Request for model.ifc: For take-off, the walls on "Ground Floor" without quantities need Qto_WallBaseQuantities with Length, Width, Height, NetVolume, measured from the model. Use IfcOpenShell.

First a look at what the model holds.

```python
import ifcopenshell
import ifcopenshell.util.element
import ifcopenshell.util.unit

model = ifcopenshell.open("model.ifc")
print(model.schema)
for unit_type in ("LENGTHUNIT", "AREAUNIT", "VOLUMEUNIT"):
    print(unit_type, ifcopenshell.util.unit.calculate_unit_scale(model, unit_type))
storey = next(s for s in model.by_type("IfcBuildingStorey") if s.Name == "Ground Floor")
walls = [e for e in ifcopenshell.util.element.get_decomposition(storey) if e.is_a("IfcWall")]
for e in sorted(walls, key=lambda e: e.id()):
    print(e.id(), e.is_a(), e.Name, list(ifcopenshell.util.element.get_psets(e, qtos_only=True)), sep=" | ")
```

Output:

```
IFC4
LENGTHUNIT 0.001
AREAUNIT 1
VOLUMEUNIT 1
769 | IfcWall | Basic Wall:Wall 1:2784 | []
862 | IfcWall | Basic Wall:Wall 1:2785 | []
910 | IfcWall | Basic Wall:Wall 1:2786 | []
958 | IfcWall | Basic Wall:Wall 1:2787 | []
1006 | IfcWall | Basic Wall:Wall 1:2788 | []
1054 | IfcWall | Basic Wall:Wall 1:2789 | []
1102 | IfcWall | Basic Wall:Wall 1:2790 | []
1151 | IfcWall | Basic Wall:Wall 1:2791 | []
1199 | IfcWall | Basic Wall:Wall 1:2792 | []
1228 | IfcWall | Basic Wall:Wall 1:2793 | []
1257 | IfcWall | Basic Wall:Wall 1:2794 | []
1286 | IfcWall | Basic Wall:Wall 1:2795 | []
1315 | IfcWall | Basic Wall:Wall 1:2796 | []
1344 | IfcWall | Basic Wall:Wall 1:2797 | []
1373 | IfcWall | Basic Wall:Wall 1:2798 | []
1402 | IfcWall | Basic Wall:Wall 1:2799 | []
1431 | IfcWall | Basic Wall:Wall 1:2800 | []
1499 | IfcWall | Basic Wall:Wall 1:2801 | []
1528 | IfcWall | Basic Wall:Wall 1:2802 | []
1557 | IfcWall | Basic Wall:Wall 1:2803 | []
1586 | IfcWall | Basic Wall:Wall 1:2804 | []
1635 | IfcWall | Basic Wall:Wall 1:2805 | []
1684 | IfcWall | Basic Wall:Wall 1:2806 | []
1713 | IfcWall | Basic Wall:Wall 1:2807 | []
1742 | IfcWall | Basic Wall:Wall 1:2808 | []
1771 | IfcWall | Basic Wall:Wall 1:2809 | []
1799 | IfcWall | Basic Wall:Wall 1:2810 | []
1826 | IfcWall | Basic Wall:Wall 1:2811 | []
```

```python
import ifcopenshell
import ifcopenshell.api.pset
import ifcopenshell.geom
import ifcopenshell.util.element
import ifcopenshell.util.shape
import ifcopenshell.util.unit

model = ifcopenshell.open("model.ifc")
unit_scale = ifcopenshell.util.unit.calculate_unit_scale(model)
volume_scale = ifcopenshell.util.unit.calculate_unit_scale(model, "VOLUMEUNIT")
settings = ifcopenshell.geom.settings()

storey = next(s for s in model.by_type("IfcBuildingStorey") if s.Name == "Ground Floor")
walls = [e for e in ifcopenshell.util.element.get_decomposition(storey) if e.is_a("IfcWall")]

for e in sorted(walls, key=lambda e: e.id()):
    if ifcopenshell.util.element.get_psets(e, qtos_only=True, should_inherit=False):
        continue
    # Geometry comes back in metres, in the element's own axes.
    shape = ifcopenshell.geom.create_shape(settings, e)
    values = {
        "Length": ifcopenshell.util.shape.get_x(shape.geometry) / unit_scale,
        "Width": ifcopenshell.util.shape.get_y(shape.geometry) / unit_scale,
        "Height": ifcopenshell.util.shape.get_z(shape.geometry) / unit_scale,
        "NetVolume": ifcopenshell.util.shape.get_volume(shape.geometry) / volume_scale,
    }
    qto = ifcopenshell.api.pset.add_qto(model, product=e, name="Qto_WallBaseQuantities")
    ifcopenshell.api.pset.edit_qto(model, qto=qto, properties=values)
    print(e.id(), {k: round(v, 3) for k, v in values.items()})

model.write("model_edited.ifc")
```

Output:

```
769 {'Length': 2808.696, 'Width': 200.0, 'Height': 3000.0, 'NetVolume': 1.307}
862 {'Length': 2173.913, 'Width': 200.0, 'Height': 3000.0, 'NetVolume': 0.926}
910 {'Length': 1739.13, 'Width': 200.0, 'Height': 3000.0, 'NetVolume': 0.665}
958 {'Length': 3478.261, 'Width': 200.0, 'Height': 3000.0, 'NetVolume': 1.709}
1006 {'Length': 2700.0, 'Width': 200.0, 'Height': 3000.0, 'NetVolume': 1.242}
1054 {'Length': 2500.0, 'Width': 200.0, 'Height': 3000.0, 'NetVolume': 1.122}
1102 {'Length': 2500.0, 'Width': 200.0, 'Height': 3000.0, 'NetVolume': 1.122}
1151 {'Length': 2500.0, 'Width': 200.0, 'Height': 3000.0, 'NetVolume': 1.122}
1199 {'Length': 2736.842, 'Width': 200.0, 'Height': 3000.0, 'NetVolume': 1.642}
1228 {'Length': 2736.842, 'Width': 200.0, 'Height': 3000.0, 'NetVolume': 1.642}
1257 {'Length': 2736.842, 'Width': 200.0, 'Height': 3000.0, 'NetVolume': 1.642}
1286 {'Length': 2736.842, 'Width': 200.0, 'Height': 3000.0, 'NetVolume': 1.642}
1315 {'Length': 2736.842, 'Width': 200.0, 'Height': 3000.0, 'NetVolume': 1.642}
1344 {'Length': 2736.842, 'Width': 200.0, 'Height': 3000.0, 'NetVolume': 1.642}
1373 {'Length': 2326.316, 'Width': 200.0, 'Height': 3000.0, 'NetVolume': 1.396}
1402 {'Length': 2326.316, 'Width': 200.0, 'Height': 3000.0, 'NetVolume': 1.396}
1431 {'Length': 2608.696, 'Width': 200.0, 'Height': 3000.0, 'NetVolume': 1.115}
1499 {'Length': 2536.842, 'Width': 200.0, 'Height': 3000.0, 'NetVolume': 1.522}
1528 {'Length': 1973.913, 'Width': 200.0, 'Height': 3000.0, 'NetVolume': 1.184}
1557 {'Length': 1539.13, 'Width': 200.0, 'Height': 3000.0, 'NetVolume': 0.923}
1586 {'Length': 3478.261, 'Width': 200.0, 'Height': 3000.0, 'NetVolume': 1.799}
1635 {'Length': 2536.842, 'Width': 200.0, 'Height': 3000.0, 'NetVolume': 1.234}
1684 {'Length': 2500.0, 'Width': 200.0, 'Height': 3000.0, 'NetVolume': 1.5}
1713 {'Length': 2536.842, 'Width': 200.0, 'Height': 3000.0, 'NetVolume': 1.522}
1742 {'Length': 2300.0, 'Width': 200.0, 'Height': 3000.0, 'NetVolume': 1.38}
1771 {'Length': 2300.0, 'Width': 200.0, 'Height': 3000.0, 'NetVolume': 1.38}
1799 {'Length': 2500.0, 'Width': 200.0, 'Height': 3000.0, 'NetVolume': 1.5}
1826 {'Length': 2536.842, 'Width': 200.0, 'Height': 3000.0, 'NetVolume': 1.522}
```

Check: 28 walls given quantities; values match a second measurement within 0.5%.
